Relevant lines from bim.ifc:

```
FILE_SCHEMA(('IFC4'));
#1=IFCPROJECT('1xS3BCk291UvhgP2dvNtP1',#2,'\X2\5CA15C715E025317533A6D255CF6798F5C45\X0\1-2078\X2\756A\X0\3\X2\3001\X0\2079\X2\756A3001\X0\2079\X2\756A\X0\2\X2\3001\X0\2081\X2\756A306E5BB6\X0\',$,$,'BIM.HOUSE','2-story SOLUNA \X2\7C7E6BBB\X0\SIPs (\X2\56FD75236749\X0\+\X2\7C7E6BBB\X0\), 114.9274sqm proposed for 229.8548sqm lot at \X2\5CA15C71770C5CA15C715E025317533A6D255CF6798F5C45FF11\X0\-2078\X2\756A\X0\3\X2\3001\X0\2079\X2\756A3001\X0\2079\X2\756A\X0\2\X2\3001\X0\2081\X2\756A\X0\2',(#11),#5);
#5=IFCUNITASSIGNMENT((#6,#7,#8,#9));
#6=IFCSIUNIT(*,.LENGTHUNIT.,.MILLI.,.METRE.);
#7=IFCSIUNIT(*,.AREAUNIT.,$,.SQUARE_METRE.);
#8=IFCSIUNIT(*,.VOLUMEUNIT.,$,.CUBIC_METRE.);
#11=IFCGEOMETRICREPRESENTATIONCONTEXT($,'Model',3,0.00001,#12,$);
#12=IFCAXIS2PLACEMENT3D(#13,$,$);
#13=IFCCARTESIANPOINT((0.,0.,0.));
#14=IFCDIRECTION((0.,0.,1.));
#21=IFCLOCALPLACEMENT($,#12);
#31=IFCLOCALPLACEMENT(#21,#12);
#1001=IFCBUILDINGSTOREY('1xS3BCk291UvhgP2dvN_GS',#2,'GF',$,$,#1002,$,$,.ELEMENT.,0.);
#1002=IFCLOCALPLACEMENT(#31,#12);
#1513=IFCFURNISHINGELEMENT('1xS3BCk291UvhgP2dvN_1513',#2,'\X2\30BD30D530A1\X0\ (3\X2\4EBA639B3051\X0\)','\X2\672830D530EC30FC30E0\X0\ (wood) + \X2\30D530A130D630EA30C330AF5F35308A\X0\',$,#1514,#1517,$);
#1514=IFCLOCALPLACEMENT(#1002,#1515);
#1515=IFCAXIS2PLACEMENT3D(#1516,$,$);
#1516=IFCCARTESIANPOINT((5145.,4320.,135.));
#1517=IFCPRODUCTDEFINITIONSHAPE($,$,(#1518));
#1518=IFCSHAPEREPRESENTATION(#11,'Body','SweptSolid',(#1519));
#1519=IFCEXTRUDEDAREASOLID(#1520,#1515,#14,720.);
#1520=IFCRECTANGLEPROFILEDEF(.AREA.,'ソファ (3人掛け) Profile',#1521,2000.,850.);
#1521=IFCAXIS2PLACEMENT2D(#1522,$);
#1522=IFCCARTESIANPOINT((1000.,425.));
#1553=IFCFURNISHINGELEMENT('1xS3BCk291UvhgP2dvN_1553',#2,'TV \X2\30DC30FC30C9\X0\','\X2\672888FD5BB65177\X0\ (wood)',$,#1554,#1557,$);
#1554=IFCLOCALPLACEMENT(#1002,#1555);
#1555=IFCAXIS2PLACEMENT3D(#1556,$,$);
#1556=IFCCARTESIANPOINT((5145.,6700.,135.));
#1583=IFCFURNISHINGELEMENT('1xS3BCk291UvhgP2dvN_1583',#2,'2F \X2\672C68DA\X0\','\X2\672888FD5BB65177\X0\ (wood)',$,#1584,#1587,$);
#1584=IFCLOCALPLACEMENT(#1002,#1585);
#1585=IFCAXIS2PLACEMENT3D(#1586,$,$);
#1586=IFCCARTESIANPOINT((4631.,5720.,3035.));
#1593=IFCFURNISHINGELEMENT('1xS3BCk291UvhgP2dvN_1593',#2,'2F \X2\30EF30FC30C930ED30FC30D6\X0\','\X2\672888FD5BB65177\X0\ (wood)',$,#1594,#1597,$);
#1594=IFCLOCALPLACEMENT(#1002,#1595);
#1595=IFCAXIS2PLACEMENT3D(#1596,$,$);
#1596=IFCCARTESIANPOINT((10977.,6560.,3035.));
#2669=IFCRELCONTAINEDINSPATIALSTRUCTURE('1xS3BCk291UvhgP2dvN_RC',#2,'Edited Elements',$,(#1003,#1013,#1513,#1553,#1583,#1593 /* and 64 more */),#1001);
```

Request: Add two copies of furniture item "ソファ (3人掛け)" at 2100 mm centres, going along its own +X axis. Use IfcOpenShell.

```python
import ifcopenshell
import ifcopenshell.api.geometry
import ifcopenshell.api.root
import ifcopenshell.util.element
import ifcopenshell.util.placement
import ifcopenshell.util.unit

model = ifcopenshell.open("bim.ifc")
unit_scale = ifcopenshell.util.unit.calculate_unit_scale(model)


def reuse_history(source, copy):
    """copy_class also copies each property set's owner history, people and application; keep the originals."""
    for rel in copy.IsDefinedBy:
        if rel.is_a("IfcRelDefinesByProperties") and (history := rel.RelatingPropertyDefinition.OwnerHistory):
            rel.RelatingPropertyDefinition.OwnerHistory = source.OwnerHistory
            ifcopenshell.util.element.remove_deep2(model, history)


source = model.by_guid("1xS3BCk291UvhgP2dvN_1513")
base = ifcopenshell.util.placement.get_local_placement(source.ObjectPlacement)
step = base[:3, 0] * 2.1 / unit_scale

for i in range(1, 3):
    copy = ifcopenshell.api.root.copy_class(model, product=source)
    copy.Representation = ifcopenshell.util.element.copy_deep(
        model, source.Representation, exclude=["IfcGeometricRepresentationContext", "IfcRepresentationMap"]
    )
    reuse_history(source, copy)
    matrix = base.copy()
    matrix[:3, 3] += i * step
    print("added at", matrix[:3, 3].round(3) + 0.0)
    ifcopenshell.api.geometry.edit_object_placement(model, product=copy, matrix=matrix, is_si=False)

model.write("bim-out.ifc")
```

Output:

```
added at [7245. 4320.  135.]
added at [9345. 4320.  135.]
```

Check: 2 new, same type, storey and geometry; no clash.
